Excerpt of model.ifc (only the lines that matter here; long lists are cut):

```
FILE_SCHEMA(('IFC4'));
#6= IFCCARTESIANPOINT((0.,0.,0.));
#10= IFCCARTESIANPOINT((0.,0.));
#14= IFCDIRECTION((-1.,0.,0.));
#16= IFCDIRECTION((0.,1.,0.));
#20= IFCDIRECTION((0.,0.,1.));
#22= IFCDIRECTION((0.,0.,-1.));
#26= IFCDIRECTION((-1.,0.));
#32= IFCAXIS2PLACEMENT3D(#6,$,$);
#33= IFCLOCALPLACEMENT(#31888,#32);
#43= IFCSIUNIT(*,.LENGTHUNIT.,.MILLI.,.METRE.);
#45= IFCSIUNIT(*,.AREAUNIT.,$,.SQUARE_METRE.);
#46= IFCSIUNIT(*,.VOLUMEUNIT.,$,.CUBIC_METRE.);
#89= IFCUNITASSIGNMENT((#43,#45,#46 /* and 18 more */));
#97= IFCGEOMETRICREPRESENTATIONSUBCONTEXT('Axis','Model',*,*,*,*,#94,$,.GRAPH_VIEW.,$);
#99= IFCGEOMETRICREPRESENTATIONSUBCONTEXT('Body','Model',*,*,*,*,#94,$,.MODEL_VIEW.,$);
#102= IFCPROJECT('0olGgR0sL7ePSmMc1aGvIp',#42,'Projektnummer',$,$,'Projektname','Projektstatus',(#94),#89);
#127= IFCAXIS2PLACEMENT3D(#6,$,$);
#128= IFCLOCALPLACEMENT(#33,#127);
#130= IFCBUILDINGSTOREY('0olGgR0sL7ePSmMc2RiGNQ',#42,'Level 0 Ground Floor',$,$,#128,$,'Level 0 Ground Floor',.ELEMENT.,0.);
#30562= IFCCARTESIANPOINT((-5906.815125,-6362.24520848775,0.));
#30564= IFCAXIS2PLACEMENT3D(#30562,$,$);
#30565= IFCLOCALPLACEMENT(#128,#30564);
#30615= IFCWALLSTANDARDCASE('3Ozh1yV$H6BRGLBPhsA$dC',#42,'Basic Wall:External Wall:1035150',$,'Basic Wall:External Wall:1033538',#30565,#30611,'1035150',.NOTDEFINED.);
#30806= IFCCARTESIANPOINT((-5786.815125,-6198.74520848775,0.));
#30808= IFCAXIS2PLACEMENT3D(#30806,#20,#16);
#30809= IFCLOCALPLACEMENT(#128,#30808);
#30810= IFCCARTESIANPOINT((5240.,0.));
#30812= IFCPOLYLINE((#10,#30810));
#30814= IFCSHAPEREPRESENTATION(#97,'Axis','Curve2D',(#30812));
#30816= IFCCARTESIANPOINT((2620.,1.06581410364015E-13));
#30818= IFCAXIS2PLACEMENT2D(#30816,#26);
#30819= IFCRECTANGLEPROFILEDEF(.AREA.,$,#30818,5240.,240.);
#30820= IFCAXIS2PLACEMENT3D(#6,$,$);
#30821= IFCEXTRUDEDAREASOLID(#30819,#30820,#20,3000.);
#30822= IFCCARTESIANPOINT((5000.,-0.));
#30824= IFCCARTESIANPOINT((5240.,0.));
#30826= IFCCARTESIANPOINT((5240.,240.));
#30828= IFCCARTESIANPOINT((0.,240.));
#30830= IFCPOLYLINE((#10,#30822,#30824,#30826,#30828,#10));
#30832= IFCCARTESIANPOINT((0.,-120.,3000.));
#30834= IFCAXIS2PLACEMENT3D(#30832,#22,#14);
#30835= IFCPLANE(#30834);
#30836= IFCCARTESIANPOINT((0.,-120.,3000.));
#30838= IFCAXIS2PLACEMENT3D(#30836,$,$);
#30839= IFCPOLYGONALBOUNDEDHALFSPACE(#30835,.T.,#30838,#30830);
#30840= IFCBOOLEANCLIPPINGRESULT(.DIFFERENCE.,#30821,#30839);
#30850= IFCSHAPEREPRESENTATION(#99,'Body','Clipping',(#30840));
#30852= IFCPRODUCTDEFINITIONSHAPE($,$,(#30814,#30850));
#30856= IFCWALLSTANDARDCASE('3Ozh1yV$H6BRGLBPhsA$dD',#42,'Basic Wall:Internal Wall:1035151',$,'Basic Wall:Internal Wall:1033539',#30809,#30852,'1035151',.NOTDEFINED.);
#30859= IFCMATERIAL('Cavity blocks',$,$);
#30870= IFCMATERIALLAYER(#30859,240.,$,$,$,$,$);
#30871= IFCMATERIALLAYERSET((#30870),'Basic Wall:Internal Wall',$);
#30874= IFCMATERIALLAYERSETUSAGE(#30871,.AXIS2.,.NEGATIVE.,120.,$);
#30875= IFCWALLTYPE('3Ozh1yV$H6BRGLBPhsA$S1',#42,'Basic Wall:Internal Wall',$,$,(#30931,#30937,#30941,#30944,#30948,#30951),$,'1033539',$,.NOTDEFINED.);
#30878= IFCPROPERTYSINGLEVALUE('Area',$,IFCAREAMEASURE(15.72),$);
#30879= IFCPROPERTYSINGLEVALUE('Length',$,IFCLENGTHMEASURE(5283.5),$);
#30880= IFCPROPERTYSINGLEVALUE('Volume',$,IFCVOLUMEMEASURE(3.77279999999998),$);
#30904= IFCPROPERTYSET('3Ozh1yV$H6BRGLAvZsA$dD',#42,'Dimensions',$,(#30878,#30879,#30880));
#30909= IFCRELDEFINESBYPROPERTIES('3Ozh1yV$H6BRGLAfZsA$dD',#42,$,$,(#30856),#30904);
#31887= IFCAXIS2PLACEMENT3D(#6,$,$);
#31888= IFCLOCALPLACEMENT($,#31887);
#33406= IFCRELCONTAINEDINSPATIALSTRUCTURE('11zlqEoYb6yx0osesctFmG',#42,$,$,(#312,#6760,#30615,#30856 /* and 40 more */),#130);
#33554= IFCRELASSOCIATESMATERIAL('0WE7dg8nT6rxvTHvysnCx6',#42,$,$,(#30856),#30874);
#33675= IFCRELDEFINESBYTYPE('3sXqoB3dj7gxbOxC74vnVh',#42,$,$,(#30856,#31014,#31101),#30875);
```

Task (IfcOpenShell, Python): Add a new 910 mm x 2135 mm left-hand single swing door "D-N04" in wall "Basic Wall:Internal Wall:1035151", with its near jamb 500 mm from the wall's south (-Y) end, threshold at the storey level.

```python
import numpy as np
import ifcopenshell
import ifcopenshell.api.feature
import ifcopenshell.api.geometry
import ifcopenshell.api.pset
import ifcopenshell.api.root
import ifcopenshell.api.spatial
import ifcopenshell.geom
import ifcopenshell.util.element
import ifcopenshell.util.placement
import ifcopenshell.util.representation
import ifcopenshell.util.shape
import ifcopenshell.util.unit

model = ifcopenshell.open("model.ifc")
unit_scale = ifcopenshell.util.unit.calculate_unit_scale(model)
area_scale = ifcopenshell.util.unit.calculate_unit_scale(model, "AREAUNIT")
volume_scale = ifcopenshell.util.unit.calculate_unit_scale(model, "VOLUMEUNIT")
settings = ifcopenshell.geom.settings()


def volume(element):
    """Net volume in cubic metres, openings subtracted."""
    shape = ifcopenshell.geom.create_shape(settings, element)
    return ifcopenshell.util.shape.get_volume(shape.geometry)


wall = model.by_id(30856)
storey = ifcopenshell.util.element.get_container(wall, ifc_class="IfcBuildingStorey")
context = ifcopenshell.util.representation.get_context(model, "Model", "Body", "MODEL_VIEW")
before = volume(wall)

width, height, from_end, sill = 0.91, 2.135, 0.5, 0.0  # metres

# The wall runs along its own X axis, and the end named is its -X end.
wall_shape = ifcopenshell.geom.create_shape(settings, wall)
x, y, z = ifcopenshell.util.shape.get_vertices(wall_shape.geometry).T
start = x.min() + from_end
face, thickness = float(y.min()), float(y.max() - y.min())
wall_matrix = ifcopenshell.util.placement.get_local_placement(wall.ObjectPlacement)
level = ifcopenshell.util.placement.get_local_placement(storey.ObjectPlacement)[2, 3]


def in_wall(x, y):
    """Placement at x, y metres in the wall's axes, at sill height."""
    matrix = wall_matrix.copy()
    matrix[:, 3] = wall_matrix @ np.array([x / unit_scale, y / unit_scale, 0.0, 1.0])
    matrix[2, 3] = level + sill / unit_scale
    return matrix


# Opening: a box that overshoots both wall faces by 50 mm.
opening = ifcopenshell.api.root.create_entity(model, ifc_class="IfcOpeningElement", predefined_type="OPENING")
box = ifcopenshell.api.geometry.add_wall_representation(
    model, context=context, length=width, height=height, thickness=thickness + 0.1
)
ifcopenshell.api.geometry.assign_representation(model, product=opening, representation=box)
ifcopenshell.api.geometry.edit_object_placement(model, product=opening, matrix=in_wall(start, face - 0.05), is_si=False)
ifcopenshell.api.feature.add_feature(model, feature=opening, element=wall)

door = ifcopenshell.api.root.create_entity(model, ifc_class="IfcDoor", name="D-N04", predefined_type="DOOR")
door.OverallWidth, door.OverallHeight = width / unit_scale, height / unit_scale
door.OperationType = "SINGLE_SWING_LEFT"
body = ifcopenshell.api.geometry.add_door_representation(
    model,
    context=context,
    overall_width=door.OverallWidth,
    overall_height=door.OverallHeight,
    operation_type="SINGLE_SWING_LEFT",
    lining_properties={"LiningDepth": thickness / unit_scale, "ThresholdDepth": thickness / unit_scale},
)
ifcopenshell.api.geometry.assign_representation(model, product=door, representation=body)
ifcopenshell.api.spatial.assign_container(model, products=[door], relating_structure=storey)
ifcopenshell.api.feature.add_filling(model, opening=opening, element=door)

# The lining spans the wall, so the door starts at the wall face.
ifcopenshell.api.geometry.edit_object_placement(model, product=door, matrix=in_wall(start, face), is_si=False)

after = volume(wall)

# Update the wall's stored quantities.
pset = model.by_id(ifcopenshell.util.element.get_pset(wall, "Dimensions", should_inherit=False)["id"])
ifcopenshell.api.pset.edit_pset(model, pset=pset, properties={
    "Area": model.create_entity("IfcAreaMeasure", after / thickness / area_scale),
    "Volume": model.create_entity("IfcVolumeMeasure", after / volume_scale),
})

print(f"wall volume {before:.3f} -> {after:.3f} m3")

model.write("model-out.ifc")
```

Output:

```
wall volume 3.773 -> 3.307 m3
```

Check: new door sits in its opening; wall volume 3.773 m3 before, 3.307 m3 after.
